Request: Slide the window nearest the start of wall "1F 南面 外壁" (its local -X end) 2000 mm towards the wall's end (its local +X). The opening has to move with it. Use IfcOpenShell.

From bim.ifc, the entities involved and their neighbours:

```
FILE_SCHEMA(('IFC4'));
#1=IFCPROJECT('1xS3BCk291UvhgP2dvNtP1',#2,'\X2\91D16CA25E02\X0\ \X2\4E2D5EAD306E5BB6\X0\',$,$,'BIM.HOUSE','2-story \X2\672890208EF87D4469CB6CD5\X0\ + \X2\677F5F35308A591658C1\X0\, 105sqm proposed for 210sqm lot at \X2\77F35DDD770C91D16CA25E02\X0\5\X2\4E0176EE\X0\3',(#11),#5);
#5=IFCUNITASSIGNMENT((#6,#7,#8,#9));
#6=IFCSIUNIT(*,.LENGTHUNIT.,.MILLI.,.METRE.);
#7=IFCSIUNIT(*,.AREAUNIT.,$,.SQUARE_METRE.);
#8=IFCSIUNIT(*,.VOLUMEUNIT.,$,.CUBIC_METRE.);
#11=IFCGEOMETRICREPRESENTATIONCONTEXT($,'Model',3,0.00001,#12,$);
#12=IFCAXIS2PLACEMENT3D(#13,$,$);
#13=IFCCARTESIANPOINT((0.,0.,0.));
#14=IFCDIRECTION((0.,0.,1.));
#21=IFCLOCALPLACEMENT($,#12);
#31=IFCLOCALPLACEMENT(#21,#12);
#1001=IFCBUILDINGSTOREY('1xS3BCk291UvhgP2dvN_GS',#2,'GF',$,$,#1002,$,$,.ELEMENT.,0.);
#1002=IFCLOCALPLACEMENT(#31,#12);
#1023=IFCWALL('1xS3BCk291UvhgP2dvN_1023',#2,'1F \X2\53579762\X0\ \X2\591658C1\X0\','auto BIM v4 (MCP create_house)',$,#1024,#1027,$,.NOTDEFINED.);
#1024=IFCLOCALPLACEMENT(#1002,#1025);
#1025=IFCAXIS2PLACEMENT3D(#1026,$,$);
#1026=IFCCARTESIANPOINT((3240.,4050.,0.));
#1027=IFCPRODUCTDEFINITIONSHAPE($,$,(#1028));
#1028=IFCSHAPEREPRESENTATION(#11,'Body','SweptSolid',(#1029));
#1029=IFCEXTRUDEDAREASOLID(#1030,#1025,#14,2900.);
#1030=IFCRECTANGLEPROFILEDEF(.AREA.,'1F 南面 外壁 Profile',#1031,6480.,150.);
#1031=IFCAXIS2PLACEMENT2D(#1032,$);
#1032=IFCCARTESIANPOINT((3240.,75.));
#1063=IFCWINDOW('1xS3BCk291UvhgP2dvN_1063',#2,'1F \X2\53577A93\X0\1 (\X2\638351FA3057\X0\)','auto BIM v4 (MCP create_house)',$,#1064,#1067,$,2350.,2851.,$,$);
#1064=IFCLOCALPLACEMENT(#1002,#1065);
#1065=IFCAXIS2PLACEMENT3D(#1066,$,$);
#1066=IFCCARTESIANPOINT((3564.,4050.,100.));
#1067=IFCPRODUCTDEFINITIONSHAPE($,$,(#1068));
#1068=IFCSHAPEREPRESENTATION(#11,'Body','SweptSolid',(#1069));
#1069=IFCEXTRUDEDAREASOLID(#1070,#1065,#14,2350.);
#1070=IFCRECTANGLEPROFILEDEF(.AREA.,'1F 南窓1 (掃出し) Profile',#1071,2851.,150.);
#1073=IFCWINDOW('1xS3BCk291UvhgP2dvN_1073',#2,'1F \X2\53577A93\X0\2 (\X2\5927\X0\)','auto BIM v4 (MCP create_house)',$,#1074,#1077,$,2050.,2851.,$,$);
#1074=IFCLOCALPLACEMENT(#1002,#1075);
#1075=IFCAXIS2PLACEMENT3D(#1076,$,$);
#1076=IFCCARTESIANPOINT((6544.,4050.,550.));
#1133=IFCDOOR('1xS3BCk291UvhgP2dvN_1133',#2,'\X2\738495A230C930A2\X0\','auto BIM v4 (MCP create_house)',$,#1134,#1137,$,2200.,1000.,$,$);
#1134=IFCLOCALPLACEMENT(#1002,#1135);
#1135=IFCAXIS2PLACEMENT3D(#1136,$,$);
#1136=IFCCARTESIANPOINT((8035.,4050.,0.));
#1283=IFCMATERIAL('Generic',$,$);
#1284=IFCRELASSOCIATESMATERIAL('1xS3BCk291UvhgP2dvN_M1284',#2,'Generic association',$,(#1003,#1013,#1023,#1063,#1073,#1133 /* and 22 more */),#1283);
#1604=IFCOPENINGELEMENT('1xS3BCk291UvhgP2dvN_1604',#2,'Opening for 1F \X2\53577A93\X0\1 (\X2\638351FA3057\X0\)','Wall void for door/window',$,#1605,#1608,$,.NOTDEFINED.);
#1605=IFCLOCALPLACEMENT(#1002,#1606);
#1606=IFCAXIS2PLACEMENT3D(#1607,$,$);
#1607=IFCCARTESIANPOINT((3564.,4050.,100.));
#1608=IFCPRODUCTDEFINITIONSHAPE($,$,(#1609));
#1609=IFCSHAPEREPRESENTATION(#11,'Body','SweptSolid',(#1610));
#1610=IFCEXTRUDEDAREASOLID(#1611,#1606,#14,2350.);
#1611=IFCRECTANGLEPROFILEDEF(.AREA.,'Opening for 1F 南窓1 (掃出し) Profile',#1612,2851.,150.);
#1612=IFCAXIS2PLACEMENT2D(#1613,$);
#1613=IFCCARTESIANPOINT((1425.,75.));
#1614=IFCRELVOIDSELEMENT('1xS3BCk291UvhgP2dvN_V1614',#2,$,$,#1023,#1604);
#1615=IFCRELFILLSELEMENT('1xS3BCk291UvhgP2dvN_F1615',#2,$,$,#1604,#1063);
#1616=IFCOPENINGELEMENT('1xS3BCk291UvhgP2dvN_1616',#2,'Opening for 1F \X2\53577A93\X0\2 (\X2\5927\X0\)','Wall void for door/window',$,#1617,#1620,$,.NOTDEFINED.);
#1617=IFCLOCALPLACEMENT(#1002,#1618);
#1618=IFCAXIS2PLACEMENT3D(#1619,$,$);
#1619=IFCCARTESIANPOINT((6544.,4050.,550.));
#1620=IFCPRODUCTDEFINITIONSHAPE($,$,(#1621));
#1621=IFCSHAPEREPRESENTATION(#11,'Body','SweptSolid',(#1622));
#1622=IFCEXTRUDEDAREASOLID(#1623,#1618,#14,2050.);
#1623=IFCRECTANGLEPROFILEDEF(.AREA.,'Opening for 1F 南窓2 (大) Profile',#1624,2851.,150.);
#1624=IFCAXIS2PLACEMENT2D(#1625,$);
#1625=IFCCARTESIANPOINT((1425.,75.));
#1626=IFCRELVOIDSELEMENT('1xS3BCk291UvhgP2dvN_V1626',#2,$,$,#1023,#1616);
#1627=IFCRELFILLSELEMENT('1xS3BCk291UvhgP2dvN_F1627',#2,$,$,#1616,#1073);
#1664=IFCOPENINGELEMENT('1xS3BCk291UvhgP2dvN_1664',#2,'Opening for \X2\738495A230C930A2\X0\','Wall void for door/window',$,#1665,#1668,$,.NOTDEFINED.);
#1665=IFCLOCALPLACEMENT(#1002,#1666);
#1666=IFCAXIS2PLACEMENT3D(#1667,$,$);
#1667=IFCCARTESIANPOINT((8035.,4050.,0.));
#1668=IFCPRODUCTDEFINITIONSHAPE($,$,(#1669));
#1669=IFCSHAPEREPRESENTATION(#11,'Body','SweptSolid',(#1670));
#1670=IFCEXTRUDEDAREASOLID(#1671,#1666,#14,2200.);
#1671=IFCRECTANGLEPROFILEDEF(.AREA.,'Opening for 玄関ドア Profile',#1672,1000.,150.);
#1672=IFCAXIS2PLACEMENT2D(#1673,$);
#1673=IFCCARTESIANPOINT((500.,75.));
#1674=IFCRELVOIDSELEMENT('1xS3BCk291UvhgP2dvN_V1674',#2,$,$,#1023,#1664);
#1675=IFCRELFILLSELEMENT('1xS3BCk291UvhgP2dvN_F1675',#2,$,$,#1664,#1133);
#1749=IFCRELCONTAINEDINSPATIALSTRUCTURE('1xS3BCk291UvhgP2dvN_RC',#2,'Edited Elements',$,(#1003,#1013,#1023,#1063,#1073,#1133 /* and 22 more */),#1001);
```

```python
import ifcopenshell
import ifcopenshell.api.geometry
import ifcopenshell.util.placement
import ifcopenshell.util.unit

model = ifcopenshell.open("bim.ifc")
unit_scale = ifcopenshell.util.unit.calculate_unit_scale(model)

window = model.by_guid("1xS3BCk291UvhgP2dvN_1063")
opening = window.FillsVoids[0].RelatingOpeningElement
wall = opening.VoidsElements[0].RelatingBuildingElement

wall_matrix = ifcopenshell.util.placement.get_local_placement(wall.ObjectPlacement)
shift = wall_matrix[:3, 0] * 2 / unit_scale
before = ifcopenshell.util.placement.get_local_placement(window.ObjectPlacement)[:3, 3].copy()

# The window is not placed relative to its opening, so move both.
for product in (opening, window):
    matrix = ifcopenshell.util.placement.get_local_placement(product.ObjectPlacement)
    matrix[:3, 3] += shift
    ifcopenshell.api.geometry.edit_object_placement(model, product=product, matrix=matrix, is_si=False)

after = ifcopenshell.util.placement.get_local_placement(window.ObjectPlacement)[:3, 3]
print("window moved by", (after - before).round(3) + 0.0)

model.write("bim_updated.ifc")
```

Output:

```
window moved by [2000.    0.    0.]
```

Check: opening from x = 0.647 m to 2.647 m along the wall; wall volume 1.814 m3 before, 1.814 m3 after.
